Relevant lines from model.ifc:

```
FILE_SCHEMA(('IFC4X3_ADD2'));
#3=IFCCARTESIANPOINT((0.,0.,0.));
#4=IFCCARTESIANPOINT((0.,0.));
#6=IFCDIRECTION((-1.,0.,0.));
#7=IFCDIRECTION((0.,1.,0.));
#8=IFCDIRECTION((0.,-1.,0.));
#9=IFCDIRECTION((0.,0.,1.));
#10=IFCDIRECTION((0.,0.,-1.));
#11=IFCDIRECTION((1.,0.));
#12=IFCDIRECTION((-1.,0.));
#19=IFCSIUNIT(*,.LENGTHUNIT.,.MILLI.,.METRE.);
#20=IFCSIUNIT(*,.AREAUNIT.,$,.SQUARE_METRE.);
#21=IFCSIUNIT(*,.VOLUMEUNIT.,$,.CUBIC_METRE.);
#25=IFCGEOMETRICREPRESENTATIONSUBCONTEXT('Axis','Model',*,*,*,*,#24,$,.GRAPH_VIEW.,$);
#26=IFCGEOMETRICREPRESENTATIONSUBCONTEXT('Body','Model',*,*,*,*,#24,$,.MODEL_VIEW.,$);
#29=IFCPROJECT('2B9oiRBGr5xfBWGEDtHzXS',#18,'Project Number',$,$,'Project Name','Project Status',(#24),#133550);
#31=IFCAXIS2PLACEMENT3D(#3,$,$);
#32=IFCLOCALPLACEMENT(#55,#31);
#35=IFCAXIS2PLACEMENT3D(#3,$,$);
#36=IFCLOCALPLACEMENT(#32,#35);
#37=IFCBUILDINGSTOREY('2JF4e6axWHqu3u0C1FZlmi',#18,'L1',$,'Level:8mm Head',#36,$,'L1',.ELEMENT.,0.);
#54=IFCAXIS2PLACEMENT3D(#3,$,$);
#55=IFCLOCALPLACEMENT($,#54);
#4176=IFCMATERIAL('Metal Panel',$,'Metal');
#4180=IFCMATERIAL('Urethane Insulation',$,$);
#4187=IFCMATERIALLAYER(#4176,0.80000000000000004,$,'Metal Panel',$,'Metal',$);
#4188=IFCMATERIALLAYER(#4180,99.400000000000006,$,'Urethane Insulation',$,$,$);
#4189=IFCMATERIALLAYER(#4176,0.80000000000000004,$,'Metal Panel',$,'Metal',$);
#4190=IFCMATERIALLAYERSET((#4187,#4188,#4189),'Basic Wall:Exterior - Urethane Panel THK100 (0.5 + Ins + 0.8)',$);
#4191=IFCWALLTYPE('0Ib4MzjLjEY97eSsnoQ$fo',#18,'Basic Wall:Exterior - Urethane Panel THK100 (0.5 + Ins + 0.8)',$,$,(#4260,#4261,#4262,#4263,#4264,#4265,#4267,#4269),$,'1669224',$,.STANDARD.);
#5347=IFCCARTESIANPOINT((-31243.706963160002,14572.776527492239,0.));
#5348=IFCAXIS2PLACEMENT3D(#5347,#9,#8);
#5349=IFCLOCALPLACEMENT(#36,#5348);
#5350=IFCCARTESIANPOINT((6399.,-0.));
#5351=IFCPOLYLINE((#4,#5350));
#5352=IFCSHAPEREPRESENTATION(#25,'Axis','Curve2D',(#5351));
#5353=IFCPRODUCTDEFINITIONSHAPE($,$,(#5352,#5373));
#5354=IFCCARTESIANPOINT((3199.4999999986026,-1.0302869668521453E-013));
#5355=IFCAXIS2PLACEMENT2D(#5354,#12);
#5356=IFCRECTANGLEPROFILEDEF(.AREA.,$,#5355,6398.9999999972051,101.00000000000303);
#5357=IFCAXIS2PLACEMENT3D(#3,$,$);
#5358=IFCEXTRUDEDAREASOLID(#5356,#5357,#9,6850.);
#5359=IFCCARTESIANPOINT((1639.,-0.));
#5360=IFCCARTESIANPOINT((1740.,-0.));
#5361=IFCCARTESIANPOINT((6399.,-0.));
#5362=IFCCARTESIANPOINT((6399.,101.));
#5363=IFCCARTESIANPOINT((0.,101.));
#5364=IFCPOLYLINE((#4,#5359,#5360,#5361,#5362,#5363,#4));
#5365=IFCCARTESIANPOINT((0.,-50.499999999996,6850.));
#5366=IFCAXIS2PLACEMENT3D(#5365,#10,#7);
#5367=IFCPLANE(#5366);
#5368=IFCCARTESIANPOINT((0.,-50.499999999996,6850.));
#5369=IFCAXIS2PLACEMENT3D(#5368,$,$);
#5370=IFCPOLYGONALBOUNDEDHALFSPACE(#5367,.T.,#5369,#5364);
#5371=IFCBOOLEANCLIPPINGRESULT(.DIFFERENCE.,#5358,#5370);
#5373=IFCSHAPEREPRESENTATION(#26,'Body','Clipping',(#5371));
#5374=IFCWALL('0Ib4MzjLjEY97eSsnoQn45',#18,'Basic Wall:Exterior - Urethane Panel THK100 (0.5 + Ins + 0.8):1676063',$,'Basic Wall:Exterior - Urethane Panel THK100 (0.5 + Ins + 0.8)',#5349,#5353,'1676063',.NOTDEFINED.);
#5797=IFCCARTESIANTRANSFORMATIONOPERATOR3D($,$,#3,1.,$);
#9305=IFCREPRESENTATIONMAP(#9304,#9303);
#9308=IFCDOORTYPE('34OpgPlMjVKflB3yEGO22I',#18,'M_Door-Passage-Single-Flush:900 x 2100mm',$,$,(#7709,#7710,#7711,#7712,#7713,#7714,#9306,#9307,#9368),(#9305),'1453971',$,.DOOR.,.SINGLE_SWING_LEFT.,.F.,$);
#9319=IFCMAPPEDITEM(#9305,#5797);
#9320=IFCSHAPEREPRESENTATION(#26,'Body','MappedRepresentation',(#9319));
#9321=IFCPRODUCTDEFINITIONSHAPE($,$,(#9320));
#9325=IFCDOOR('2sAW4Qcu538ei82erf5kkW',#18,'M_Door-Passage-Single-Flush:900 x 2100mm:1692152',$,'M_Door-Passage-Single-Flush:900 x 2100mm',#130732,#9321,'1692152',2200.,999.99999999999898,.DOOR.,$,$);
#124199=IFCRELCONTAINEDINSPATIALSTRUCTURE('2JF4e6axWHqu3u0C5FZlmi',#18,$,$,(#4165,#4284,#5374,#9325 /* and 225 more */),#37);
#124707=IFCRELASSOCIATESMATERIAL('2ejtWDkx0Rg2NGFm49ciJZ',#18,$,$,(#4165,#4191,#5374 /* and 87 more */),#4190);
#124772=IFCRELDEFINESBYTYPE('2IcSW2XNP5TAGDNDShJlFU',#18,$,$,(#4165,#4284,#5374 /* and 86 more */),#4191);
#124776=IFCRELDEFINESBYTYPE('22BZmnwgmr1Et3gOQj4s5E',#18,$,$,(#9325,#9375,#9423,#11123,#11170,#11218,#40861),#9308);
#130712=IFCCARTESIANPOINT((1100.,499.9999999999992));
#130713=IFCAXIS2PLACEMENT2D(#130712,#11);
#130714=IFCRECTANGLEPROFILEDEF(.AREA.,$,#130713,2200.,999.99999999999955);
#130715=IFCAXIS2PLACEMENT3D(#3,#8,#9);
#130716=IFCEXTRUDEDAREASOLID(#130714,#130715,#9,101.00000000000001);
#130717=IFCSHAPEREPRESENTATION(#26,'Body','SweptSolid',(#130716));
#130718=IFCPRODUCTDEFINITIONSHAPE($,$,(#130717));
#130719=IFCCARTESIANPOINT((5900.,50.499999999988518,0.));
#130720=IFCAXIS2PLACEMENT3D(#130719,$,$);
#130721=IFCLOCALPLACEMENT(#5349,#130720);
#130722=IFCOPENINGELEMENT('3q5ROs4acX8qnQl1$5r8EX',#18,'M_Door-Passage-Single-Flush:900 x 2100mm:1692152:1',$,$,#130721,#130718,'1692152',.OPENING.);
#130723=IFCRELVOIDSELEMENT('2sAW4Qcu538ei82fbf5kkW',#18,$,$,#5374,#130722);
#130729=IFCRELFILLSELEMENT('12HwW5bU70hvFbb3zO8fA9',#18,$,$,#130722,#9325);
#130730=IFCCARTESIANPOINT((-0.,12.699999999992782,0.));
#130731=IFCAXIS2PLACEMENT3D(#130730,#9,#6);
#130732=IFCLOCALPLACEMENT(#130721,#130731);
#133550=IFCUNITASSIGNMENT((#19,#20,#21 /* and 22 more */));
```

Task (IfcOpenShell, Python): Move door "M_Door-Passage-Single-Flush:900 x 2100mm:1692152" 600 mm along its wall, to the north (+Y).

```python
import ifcopenshell
import ifcopenshell.api.geometry
import ifcopenshell.util.placement
import ifcopenshell.util.unit

model = ifcopenshell.open("model.ifc")
unit_scale = ifcopenshell.util.unit.calculate_unit_scale(model)

door = model.by_id(9325)
opening = door.FillsVoids[0].RelatingOpeningElement
wall = opening.VoidsElements[0].RelatingBuildingElement

wall_matrix = ifcopenshell.util.placement.get_local_placement(wall.ObjectPlacement)
shift = wall_matrix[:3, 0] * -0.6 / unit_scale
before = ifcopenshell.util.placement.get_local_placement(door.ObjectPlacement)[:3, 3].copy()

# The door is placed relative to its opening, so it follows when the opening moves.
matrix = ifcopenshell.util.placement.get_local_placement(opening.ObjectPlacement)
matrix[:3, 3] += shift
ifcopenshell.api.geometry.edit_object_placement(
    model, product=opening, matrix=matrix, is_si=False, should_transform_children=True
)

after = ifcopenshell.util.placement.get_local_placement(door.ObjectPlacement)[:3, 3]
print("door moved by", (after - before).round(3) + 0.0)

model.write("model_v2.ifc")
```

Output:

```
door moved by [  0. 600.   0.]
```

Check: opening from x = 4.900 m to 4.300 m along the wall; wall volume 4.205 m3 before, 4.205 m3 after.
